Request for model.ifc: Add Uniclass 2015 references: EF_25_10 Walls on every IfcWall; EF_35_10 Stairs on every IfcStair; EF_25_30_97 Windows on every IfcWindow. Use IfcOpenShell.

First a look at what the model holds.

```python
import ifcopenshell

model = ifcopenshell.open("model.ifc")
print(model.schema)
print("classifications:", [c.Name for c in model.by_type("IfcClassification")])
for ifc_class in ("IfcDoor", "IfcRoof", "IfcStair", "IfcWall", "IfcWindow"):
    print(ifc_class, len(model.by_type(ifc_class)))
```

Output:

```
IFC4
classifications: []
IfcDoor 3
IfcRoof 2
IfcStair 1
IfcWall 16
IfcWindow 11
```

```python
import ifcopenshell
import ifcopenshell.api.classification

model = ifcopenshell.open("model.ifc")

system = ifcopenshell.api.classification.add_classification(model, classification="Uniclass 2015")

codes = {
    "IfcWall": ("EF_25_10", "Walls"),
    "IfcStair": ("EF_35_10", "Stairs"),
    "IfcWindow": ("EF_25_30_97", "Windows"),
}
for ifc_class, (code, name) in codes.items():
    products = model.by_type(ifc_class)
    ifcopenshell.api.classification.add_reference(
        model, products=products, classification=system, identification=code, name=name
    )
    print(code, len(products))

model.write("model_updated.ifc")
```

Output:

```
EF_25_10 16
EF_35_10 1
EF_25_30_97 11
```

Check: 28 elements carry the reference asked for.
